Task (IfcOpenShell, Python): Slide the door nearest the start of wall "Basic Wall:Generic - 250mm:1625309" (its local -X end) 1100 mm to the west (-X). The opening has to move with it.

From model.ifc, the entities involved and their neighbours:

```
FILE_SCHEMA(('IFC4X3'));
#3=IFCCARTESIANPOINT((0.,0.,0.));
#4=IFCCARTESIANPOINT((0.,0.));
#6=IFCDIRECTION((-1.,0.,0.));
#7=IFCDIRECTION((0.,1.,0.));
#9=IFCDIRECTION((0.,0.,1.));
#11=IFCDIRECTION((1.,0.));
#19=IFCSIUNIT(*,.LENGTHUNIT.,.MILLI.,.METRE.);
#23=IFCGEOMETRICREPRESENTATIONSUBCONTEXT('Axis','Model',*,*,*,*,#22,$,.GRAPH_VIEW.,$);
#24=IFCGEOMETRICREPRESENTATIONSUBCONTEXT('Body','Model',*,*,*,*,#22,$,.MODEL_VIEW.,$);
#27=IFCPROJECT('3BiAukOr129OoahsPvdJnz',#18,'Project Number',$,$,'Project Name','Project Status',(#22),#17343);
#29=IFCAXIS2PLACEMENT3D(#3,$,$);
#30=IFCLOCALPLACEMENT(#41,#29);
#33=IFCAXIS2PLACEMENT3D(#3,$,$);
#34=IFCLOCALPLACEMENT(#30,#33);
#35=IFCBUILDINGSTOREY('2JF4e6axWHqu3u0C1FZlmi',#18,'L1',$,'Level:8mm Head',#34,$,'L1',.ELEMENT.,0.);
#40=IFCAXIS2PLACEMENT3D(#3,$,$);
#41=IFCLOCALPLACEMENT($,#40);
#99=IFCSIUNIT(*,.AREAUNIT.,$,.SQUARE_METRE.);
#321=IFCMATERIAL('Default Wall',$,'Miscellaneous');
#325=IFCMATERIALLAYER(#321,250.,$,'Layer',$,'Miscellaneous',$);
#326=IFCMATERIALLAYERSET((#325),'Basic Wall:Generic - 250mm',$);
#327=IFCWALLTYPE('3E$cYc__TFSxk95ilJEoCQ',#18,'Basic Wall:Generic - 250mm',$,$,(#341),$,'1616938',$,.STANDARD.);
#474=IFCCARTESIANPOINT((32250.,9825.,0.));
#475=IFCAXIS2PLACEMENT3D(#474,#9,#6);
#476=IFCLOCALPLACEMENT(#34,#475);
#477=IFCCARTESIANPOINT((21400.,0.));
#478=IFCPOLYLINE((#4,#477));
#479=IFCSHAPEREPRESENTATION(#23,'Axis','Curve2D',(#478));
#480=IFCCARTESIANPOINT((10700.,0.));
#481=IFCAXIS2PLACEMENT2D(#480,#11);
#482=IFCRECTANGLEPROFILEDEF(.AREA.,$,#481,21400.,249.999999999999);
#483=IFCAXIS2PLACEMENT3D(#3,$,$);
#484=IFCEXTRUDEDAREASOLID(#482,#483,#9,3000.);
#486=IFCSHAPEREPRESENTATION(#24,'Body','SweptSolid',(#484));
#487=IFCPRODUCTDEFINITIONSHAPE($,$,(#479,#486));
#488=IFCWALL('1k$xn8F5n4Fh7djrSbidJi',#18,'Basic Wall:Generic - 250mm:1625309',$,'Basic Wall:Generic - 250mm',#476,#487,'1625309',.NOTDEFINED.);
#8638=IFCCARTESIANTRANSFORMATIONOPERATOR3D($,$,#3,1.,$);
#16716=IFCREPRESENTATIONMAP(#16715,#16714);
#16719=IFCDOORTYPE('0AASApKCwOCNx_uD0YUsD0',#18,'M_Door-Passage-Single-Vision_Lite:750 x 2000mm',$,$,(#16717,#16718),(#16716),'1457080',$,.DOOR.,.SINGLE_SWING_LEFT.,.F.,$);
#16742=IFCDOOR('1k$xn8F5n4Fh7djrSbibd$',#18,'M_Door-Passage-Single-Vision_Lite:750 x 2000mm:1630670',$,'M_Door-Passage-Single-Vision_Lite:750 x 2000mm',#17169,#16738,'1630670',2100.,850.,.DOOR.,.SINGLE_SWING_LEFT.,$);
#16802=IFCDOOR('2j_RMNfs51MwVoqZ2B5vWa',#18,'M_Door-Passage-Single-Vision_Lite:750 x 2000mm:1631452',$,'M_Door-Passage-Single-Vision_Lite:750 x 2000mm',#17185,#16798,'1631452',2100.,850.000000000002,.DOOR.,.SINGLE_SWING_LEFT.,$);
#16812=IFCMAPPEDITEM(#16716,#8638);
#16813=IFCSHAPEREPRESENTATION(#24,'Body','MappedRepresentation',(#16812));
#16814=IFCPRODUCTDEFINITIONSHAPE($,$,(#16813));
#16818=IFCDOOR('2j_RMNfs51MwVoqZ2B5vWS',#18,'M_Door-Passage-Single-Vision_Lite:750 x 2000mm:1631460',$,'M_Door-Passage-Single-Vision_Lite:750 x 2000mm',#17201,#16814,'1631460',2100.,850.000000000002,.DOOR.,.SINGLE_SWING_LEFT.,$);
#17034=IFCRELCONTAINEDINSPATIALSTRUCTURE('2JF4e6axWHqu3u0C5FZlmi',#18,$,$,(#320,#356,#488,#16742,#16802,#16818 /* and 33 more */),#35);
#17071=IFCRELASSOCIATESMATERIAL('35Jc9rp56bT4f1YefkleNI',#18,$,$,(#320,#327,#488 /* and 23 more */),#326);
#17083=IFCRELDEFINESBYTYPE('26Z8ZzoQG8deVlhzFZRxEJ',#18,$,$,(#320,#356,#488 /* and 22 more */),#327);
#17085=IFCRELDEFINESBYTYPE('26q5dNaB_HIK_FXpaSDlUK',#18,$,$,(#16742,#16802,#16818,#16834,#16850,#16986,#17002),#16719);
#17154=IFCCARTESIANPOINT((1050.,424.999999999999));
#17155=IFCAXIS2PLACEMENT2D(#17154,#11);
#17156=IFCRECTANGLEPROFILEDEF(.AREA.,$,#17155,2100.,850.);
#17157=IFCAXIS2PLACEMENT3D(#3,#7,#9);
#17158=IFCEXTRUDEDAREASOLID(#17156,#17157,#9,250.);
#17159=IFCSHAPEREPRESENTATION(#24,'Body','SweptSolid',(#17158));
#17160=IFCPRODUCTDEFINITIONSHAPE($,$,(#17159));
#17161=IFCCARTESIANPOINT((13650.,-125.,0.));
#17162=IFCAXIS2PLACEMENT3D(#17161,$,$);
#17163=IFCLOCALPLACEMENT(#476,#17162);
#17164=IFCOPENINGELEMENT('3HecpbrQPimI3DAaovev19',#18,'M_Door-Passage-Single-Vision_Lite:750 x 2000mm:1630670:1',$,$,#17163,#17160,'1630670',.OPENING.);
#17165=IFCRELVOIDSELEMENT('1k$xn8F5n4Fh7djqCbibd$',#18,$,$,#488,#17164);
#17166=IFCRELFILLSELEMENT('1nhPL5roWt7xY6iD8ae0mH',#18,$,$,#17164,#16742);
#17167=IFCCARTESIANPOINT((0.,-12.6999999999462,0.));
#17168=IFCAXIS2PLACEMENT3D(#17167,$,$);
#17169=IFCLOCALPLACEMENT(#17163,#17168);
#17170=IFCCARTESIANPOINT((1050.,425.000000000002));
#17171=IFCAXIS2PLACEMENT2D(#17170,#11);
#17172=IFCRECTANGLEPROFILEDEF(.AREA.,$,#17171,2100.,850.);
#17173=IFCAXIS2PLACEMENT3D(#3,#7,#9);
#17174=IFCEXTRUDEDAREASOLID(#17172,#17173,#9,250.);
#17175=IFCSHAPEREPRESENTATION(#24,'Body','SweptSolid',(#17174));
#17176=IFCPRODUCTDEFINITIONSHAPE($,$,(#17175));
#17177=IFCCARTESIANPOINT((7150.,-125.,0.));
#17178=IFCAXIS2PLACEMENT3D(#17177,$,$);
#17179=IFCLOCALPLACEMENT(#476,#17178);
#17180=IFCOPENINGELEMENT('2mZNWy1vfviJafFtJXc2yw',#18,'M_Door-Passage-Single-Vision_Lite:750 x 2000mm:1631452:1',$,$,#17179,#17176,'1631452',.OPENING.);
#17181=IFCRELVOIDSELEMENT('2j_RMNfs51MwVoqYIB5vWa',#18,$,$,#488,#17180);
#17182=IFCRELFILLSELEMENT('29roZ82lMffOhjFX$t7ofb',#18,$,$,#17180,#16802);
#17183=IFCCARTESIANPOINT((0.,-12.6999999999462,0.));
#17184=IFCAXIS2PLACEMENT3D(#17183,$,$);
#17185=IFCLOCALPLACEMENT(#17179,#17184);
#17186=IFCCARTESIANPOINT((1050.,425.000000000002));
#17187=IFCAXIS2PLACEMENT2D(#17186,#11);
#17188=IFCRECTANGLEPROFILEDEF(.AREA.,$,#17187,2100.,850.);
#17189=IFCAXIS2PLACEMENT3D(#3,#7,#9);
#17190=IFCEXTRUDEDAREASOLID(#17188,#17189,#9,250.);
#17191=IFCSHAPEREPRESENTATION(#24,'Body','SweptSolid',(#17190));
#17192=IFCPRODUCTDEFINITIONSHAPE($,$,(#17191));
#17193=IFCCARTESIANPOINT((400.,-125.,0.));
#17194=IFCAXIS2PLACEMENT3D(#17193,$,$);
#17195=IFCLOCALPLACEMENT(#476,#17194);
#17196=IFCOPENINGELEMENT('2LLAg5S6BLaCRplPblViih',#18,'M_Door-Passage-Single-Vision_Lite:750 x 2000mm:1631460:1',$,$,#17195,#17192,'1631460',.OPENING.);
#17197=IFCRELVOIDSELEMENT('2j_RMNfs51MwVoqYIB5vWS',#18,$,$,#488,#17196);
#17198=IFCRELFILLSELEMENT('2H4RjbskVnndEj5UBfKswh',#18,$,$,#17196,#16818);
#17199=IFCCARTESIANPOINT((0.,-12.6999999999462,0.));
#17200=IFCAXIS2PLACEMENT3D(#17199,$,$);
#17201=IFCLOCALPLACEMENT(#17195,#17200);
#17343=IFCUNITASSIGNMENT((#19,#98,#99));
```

```python
import ifcopenshell
import ifcopenshell.api.geometry
import ifcopenshell.util.placement
import ifcopenshell.util.unit

model = ifcopenshell.open("model.ifc")
unit_scale = ifcopenshell.util.unit.calculate_unit_scale(model)

door = model.by_id(16818)
opening = door.FillsVoids[0].RelatingOpeningElement
wall = opening.VoidsElements[0].RelatingBuildingElement

wall_matrix = ifcopenshell.util.placement.get_local_placement(wall.ObjectPlacement)
shift = wall_matrix[:3, 0] * 1.1 / unit_scale
before = ifcopenshell.util.placement.get_local_placement(door.ObjectPlacement)[:3, 3].copy()

# The door is placed relative to its opening, so it follows when the opening moves.
matrix = ifcopenshell.util.placement.get_local_placement(opening.ObjectPlacement)
matrix[:3, 3] += shift
ifcopenshell.api.geometry.edit_object_placement(
    model, product=opening, matrix=matrix, is_si=False, should_transform_children=True
)

after = ifcopenshell.util.placement.get_local_placement(door.ObjectPlacement)[:3, 3]
print("door moved by", (after - before).round(3) + 0.0)

model.write("model-out.ifc")
```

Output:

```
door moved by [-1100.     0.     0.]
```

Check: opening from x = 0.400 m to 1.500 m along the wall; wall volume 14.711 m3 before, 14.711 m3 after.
